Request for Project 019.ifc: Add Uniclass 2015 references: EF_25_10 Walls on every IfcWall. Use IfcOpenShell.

First a look at what the model holds.

```python
import ifcopenshell

model = ifcopenshell.open("Project 019.ifc")
print(model.schema)
print("classifications:", [c.Name for c in model.by_type("IfcClassification")])
for ifc_class in ("IfcDoor", "IfcRoof", "IfcStair", "IfcWall", "IfcWindow"):
    print(ifc_class, len(model.by_type(ifc_class)))
```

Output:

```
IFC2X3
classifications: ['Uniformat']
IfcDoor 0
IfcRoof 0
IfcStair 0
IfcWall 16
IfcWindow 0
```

```python
import ifcopenshell
import ifcopenshell.api.classification

model = ifcopenshell.open("Project 019.ifc")

# IFC2X3 requires Source and Edition and has no link from the project to the system.
system = model.create_entity("IfcClassification", Source="NBS", Edition="2015", Name="Uniclass 2015")

codes = {
    "IfcWall": ("EF_25_10", "Walls"),
}
for ifc_class, (code, name) in codes.items():
    products = model.by_type(ifc_class)
    ifcopenshell.api.classification.add_reference(
        model, products=products, classification=system, identification=code, name=name
    )
    print(code, len(products))

model.write("Project 019_rev.ifc")
```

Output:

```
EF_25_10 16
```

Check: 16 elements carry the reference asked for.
